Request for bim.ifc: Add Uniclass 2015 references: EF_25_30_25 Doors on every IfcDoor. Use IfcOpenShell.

First a look at what the model holds.

```python
import ifcopenshell

model = ifcopenshell.open("bim.ifc")
print(model.schema)
print("classifications:", [c.Name for c in model.by_type("IfcClassification")])
for ifc_class in ("IfcDoor", "IfcRoof", "IfcStair", "IfcWall", "IfcWindow"):
    print(ifc_class, len(model.by_type(ifc_class)))
```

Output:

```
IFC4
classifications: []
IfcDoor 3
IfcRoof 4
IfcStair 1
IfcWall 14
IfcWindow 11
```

```python
import ifcopenshell
import ifcopenshell.api.classification

model = ifcopenshell.open("bim.ifc")

system = ifcopenshell.api.classification.add_classification(model, classification="Uniclass 2015")

codes = {
    "IfcDoor": ("EF_25_30_25", "Doors"),
}
for ifc_class, (code, name) in codes.items():
    products = model.by_type(ifc_class)
    ifcopenshell.api.classification.add_reference(
        model, products=products, classification=system, identification=code, name=name
    )
    print(code, len(products))

model.write("bim_rev.ifc")
```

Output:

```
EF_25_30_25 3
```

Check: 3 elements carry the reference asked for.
